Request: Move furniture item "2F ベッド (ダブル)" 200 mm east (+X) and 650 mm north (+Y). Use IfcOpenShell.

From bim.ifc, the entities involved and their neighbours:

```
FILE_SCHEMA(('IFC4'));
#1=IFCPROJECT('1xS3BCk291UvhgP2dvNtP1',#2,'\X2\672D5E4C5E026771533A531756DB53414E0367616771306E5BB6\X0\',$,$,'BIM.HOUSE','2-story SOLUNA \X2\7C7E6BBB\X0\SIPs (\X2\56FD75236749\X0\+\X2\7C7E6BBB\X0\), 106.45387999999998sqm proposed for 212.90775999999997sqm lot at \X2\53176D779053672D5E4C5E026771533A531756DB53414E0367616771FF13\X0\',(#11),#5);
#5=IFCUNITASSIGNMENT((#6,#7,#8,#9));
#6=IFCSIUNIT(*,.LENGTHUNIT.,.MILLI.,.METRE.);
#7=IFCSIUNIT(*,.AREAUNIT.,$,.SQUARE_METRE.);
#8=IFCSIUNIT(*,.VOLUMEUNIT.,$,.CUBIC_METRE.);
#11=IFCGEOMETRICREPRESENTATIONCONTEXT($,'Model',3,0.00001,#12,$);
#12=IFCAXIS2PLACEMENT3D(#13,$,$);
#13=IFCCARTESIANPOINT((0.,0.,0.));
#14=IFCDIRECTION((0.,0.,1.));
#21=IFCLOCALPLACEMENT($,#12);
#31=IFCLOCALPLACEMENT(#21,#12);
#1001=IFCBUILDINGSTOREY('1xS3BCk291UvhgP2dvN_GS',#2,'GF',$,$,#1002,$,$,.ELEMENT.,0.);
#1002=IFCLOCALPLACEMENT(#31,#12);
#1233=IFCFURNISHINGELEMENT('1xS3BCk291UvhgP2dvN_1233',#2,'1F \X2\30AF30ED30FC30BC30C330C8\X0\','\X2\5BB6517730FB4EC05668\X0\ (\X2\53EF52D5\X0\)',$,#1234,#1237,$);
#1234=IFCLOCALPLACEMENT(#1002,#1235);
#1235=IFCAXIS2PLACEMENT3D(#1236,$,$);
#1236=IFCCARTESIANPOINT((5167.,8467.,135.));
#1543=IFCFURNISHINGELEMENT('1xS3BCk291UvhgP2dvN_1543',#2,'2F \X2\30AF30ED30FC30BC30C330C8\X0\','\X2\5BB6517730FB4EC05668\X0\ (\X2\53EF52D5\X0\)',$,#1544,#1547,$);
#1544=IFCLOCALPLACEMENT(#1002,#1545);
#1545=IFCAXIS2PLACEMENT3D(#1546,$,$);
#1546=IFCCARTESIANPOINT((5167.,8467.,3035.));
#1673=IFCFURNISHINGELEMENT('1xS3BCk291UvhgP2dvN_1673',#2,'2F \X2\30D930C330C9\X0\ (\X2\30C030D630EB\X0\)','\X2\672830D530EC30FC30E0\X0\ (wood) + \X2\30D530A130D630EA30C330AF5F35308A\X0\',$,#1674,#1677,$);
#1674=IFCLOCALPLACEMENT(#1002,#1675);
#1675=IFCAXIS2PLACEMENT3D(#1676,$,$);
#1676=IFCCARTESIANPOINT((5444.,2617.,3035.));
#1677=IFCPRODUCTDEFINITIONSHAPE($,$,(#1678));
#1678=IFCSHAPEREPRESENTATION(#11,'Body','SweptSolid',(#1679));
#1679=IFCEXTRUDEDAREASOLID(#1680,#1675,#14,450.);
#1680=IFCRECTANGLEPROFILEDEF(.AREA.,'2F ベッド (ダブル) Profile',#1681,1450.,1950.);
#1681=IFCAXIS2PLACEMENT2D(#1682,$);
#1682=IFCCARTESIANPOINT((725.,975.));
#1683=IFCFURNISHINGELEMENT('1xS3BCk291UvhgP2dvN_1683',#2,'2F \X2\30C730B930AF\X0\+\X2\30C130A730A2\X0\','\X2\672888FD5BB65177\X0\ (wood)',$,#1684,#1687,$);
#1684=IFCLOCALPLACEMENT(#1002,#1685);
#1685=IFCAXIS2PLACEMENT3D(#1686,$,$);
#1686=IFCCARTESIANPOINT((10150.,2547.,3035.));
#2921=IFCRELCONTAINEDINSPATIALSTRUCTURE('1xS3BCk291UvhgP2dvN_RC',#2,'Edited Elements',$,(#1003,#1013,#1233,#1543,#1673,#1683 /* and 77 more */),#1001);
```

```python
import ifcopenshell
import ifcopenshell.api.geometry
import ifcopenshell.util.placement
import ifcopenshell.util.unit

model = ifcopenshell.open("bim.ifc")
unit_scale = ifcopenshell.util.unit.calculate_unit_scale(model)

item = model.by_guid("1xS3BCk291UvhgP2dvN_1673")
matrix = ifcopenshell.util.placement.get_local_placement(item.ObjectPlacement)
matrix[0, 3] += 0.2 / unit_scale
matrix[1, 3] += 0.65 / unit_scale
ifcopenshell.api.geometry.edit_object_placement(model, product=item, matrix=matrix, is_si=False)

print(ifcopenshell.util.placement.get_local_placement(item.ObjectPlacement).round(3) + 0.0)

model.write("bim_v2.ifc")
```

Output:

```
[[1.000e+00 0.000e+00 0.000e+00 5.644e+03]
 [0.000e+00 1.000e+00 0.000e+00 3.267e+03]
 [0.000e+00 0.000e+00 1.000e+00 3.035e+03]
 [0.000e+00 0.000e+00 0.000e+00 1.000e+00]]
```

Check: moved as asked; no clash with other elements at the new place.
